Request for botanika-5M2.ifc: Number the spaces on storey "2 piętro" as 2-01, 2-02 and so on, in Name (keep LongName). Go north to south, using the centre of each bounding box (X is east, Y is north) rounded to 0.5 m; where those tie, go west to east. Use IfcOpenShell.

First a look at what the model holds.

```python
import ifcopenshell
import ifcopenshell.util.element
import ifcopenshell.util.placement

model = ifcopenshell.open("botanika-5M2.ifc")
print(model.schema)
storey = next(s for s in model.by_type("IfcBuildingStorey") if s.Name == "2 piętro")
spaces = [e for e in ifcopenshell.util.element.get_decomposition(storey) if e.is_a("IfcSpace")]
for e in sorted(spaces, key=lambda e: e.id()):
    origin = ifcopenshell.util.placement.get_local_placement(e.ObjectPlacement)[:3, 3]
    print(e.id(), e.Name, e.LongName, origin.round(2) + 0.0, sep=" | ")
```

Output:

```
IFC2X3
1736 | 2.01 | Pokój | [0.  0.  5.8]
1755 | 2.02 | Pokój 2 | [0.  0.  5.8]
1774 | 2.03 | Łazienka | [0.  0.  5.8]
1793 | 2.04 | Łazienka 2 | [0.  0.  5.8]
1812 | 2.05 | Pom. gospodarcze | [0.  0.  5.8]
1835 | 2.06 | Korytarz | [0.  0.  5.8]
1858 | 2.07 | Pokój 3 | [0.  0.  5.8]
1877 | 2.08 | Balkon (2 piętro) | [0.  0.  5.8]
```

```python
import ifcopenshell
import ifcopenshell.geom
import ifcopenshell.util.element
import ifcopenshell.util.shape

model = ifcopenshell.open("botanika-5M2.ifc")
settings = ifcopenshell.geom.settings()
settings.set("use-world-coords", True)


def centre(element):
    shape = ifcopenshell.geom.create_shape(settings, element)
    return ifcopenshell.util.shape.get_bbox_centroid(shape.geometry)


storey = next(s for s in model.by_type("IfcBuildingStorey") if s.Name == "2 piętro")
spaces = [e for e in ifcopenshell.util.element.get_decomposition(storey) if e.is_a("IfcSpace")]

# Insertion points can sit at a corner or the storey origin, so sort by the geometry (in metres).
centres = {e: centre(e) for e in spaces}
spaces.sort(key=lambda e: (-round(centres[e][1] / 0.5), centres[e][0]))

for i, e in enumerate(spaces, start=1):
    number = f"2-{i:02d}"
    e.Name = number
    print(e.id(), number)

model.write("botanika-5M2_updated.ifc")
```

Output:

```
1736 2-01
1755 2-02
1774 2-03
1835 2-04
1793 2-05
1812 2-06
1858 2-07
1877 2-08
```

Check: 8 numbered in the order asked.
